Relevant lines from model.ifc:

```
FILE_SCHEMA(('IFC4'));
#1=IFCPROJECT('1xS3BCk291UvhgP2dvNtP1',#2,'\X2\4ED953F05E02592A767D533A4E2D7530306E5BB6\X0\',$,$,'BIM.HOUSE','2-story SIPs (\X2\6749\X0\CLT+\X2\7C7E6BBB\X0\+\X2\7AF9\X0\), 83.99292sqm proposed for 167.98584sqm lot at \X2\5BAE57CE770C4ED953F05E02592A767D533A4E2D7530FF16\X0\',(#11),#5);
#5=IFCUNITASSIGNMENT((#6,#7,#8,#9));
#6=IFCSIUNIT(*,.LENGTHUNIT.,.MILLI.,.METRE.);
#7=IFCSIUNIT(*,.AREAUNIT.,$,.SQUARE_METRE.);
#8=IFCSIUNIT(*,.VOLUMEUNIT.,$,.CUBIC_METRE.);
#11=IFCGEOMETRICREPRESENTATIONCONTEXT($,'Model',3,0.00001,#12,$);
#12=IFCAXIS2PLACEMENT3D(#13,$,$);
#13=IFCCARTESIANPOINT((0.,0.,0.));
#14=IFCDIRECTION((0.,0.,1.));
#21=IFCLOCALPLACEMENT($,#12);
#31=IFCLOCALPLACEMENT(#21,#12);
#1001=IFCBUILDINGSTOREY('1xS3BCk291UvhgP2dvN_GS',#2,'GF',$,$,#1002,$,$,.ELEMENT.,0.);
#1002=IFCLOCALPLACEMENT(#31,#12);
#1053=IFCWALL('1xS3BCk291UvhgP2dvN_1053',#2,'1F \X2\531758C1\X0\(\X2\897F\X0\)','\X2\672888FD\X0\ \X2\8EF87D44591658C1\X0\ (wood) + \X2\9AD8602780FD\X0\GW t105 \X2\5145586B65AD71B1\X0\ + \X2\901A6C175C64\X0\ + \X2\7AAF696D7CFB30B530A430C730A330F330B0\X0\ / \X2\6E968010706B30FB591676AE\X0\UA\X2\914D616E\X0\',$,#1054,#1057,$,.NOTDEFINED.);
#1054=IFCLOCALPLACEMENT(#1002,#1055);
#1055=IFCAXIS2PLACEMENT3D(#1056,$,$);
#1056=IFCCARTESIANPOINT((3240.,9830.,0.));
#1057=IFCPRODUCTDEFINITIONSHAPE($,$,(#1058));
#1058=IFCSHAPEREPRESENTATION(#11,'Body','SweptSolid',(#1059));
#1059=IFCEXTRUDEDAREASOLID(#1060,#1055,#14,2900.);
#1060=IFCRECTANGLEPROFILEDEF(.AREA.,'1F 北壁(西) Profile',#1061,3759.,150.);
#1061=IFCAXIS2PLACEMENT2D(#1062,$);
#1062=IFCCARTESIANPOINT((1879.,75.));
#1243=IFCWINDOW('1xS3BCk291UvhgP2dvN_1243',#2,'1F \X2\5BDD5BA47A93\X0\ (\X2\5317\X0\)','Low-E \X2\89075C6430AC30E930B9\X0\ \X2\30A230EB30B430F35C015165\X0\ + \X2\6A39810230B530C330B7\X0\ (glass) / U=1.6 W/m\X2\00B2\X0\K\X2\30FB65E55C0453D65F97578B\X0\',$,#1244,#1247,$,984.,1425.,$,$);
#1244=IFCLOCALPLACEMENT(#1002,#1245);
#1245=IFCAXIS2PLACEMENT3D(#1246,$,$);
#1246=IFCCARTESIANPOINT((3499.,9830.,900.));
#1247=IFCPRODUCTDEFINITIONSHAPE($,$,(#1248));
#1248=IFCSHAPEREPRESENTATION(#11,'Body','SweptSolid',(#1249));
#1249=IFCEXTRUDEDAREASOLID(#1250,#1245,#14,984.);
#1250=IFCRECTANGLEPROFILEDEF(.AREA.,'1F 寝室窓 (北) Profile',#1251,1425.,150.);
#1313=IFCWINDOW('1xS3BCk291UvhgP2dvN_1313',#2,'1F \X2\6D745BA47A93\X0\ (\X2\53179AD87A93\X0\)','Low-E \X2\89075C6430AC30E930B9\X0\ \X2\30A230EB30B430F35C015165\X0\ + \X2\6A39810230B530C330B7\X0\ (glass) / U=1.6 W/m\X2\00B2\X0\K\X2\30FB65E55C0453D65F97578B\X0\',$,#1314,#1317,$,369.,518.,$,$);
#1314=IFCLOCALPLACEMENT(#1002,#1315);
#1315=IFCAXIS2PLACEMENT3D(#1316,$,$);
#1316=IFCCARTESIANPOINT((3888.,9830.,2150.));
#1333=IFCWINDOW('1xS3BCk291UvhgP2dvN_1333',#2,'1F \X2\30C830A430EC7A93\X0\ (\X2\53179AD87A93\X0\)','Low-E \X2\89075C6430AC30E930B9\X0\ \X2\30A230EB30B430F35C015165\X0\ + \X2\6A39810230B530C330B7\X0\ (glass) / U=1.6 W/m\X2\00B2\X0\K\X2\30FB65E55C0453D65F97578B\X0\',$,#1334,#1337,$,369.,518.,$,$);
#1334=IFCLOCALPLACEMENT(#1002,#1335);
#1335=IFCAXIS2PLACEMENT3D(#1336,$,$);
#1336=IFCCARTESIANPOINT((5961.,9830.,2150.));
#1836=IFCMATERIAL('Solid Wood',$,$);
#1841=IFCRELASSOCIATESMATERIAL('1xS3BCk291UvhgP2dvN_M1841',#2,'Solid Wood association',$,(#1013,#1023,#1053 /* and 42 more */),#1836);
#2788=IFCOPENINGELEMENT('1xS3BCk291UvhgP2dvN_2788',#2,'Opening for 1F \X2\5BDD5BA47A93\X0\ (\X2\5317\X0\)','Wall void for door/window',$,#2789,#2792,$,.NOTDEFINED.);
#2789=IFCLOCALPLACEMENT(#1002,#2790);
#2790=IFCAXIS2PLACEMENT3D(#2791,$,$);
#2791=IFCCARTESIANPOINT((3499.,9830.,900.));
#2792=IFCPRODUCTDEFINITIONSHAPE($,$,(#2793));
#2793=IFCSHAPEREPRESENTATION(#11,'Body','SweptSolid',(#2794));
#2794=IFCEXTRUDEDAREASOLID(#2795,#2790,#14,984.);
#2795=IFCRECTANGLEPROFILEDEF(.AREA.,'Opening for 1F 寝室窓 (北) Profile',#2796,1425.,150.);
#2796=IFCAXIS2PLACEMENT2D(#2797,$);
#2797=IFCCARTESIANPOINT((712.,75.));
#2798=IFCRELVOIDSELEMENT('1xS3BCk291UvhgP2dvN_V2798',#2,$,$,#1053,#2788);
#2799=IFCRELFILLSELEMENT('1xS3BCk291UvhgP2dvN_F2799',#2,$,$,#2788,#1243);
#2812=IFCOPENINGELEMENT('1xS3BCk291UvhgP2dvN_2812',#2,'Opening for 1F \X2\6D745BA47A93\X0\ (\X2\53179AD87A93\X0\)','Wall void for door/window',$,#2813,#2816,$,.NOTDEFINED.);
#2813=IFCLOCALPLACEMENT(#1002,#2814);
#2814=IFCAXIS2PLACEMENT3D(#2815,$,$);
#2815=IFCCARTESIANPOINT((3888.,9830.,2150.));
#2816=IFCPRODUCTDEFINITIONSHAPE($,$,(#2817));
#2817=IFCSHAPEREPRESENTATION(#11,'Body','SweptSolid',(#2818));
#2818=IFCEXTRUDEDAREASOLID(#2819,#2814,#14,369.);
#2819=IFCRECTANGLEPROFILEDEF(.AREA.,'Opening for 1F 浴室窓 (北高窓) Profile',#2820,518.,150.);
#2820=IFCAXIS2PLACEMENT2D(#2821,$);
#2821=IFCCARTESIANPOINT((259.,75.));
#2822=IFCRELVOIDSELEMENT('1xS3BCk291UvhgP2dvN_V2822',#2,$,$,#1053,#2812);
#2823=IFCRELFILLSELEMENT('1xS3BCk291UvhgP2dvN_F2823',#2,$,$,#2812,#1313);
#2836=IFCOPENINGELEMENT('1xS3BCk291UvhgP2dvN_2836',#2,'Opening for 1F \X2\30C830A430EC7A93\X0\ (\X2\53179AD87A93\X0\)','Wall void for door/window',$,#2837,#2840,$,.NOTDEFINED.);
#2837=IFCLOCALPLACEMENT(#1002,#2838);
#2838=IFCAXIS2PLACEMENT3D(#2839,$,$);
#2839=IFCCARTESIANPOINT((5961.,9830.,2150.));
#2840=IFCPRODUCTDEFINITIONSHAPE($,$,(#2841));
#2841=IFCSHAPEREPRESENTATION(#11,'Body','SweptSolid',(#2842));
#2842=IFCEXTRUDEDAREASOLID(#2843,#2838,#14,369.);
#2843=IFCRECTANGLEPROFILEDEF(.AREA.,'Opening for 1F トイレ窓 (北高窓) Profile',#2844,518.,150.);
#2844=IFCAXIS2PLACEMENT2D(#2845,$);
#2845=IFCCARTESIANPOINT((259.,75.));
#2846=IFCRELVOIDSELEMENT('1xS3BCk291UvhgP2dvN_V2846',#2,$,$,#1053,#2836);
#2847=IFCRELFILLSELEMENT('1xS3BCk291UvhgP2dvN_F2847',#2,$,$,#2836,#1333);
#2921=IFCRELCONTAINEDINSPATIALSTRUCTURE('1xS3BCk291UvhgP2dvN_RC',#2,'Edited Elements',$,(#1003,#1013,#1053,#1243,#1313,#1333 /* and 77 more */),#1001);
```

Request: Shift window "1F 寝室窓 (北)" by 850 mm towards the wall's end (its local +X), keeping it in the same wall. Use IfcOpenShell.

```python
import ifcopenshell
import ifcopenshell.api.geometry
import ifcopenshell.util.placement

model = ifcopenshell.open("model.ifc")

window = model.by_guid("1xS3BCk291UvhgP2dvN_1243")
opening = window.FillsVoids[0].RelatingOpeningElement
wall = opening.VoidsElements[0].RelatingBuildingElement

wall_matrix = ifcopenshell.util.placement.get_local_placement(wall.ObjectPlacement)
shift = wall_matrix[:3, 0] * 850.0
before = ifcopenshell.util.placement.get_local_placement(window.ObjectPlacement)[:3, 3].copy()

# The window is not placed relative to its opening, so move both.
for product in (opening, window):
    matrix = ifcopenshell.util.placement.get_local_placement(product.ObjectPlacement)
    matrix[:3, 3] += shift
    ifcopenshell.api.geometry.edit_object_placement(model, product=product, matrix=matrix, is_si=False)

after = ifcopenshell.util.placement.get_local_placement(window.ObjectPlacement)[:3, 3]
print("window moved by", (after - before).round(3) + 0.0)

model.write("model_v2.ifc")
```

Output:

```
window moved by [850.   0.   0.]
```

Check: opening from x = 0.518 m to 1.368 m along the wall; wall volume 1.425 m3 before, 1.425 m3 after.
